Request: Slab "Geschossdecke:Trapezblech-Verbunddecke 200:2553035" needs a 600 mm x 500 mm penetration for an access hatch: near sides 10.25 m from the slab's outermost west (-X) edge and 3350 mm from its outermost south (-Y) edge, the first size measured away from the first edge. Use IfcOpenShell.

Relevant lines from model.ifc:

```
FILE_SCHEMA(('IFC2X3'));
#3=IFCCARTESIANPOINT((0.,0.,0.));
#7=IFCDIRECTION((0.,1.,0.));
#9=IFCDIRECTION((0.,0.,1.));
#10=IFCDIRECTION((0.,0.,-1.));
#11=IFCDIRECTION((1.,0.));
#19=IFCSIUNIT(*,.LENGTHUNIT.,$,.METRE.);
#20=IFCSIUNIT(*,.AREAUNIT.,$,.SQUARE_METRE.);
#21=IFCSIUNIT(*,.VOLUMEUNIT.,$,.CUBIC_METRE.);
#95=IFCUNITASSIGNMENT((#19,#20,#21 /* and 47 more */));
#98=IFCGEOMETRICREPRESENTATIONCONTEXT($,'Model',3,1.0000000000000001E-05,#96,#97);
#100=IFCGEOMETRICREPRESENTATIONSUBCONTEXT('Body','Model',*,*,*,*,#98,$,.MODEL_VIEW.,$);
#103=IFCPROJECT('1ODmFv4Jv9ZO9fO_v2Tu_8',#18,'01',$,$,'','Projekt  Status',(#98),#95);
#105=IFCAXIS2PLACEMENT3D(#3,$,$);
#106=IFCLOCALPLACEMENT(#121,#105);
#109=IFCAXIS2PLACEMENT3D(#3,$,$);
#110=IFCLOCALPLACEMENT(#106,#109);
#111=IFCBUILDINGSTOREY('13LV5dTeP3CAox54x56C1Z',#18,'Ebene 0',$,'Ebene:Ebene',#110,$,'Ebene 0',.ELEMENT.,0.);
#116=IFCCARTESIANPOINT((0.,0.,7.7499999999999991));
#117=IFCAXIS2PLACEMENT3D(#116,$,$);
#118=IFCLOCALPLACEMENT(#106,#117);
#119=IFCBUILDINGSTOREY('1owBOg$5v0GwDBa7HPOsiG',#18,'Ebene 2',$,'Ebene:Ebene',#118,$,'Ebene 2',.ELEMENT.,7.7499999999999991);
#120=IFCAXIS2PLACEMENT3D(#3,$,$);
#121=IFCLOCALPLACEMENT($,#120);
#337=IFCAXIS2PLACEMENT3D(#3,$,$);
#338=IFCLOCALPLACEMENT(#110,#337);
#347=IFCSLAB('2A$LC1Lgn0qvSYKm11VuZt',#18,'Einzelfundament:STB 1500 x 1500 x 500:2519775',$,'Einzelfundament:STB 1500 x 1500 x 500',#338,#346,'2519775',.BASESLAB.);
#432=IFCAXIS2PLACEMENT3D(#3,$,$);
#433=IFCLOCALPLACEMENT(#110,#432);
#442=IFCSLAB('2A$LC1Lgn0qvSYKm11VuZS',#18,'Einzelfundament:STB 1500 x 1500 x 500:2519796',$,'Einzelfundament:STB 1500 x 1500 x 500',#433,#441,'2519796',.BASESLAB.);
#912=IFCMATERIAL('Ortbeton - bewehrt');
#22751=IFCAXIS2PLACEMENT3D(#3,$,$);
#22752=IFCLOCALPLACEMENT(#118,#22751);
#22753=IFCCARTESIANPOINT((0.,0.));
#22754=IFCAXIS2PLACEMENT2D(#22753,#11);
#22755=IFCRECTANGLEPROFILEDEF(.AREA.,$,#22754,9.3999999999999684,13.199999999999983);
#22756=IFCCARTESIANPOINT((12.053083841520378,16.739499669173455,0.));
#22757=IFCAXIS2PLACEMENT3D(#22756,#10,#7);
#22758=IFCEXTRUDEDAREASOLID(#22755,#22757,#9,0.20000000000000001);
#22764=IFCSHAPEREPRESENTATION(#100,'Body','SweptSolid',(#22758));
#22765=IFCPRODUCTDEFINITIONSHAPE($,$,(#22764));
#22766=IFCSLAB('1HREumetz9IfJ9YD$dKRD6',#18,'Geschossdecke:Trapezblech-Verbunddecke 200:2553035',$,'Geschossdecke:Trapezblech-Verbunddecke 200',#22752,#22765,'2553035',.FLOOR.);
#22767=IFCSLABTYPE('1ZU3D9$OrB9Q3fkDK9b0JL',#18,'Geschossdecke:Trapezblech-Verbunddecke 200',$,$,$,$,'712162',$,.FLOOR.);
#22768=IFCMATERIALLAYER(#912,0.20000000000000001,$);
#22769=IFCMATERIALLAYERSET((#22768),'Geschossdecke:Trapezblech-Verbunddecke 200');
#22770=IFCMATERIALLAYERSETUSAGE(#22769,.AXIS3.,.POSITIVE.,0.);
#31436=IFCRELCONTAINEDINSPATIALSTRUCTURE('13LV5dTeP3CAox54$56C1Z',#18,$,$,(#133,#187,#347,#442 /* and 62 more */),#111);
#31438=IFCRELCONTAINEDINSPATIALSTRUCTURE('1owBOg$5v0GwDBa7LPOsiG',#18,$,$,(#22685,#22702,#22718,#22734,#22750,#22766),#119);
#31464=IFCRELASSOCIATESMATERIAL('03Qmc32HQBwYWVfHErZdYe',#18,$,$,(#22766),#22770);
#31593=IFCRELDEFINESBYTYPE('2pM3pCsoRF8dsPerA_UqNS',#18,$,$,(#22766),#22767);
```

```python
import numpy as np
import ifcopenshell
import ifcopenshell.api.feature
import ifcopenshell.api.geometry
import ifcopenshell.api.root
import ifcopenshell.geom
import ifcopenshell.util.placement
import ifcopenshell.util.representation
import ifcopenshell.util.shape
import ifcopenshell.util.unit

model = ifcopenshell.open("model.ifc")
unit_scale = ifcopenshell.util.unit.calculate_unit_scale(model)
settings = ifcopenshell.geom.settings()


def volume(element):
    """Net volume in cubic metres, openings subtracted."""
    shape = ifcopenshell.geom.create_shape(settings, element)
    return ifcopenshell.util.shape.get_volume(shape.geometry)


slab = model.by_guid("1HREumetz9IfJ9YD$dKRD6")
before = volume(slab)

# Extent in the slab's own axes, in metres. The edges named are its -X and -Y sides.
slab_shape = ifcopenshell.geom.create_shape(settings, slab)
vertices = ifcopenshell.util.shape.get_vertices(slab_shape.geometry)
x_min, y_min, bottom = vertices.min(axis=0)
top = vertices[:, 2].max()

opening = ifcopenshell.api.root.create_entity(model, ifc_class="IfcOpeningElement", name="Access hatch opening")
context = ifcopenshell.util.representation.get_context(model, "Model", "Body", "MODEL_VIEW")
width, depth = 0.6, 0.5
outline = [(0.0, 0.0), (width, 0.0), (width, depth), (0.0, depth), (0.0, 0.0)]
# Overshoot both faces by 50 mm so the cut is clean.
shape = ifcopenshell.api.geometry.add_slab_representation(
    model, context=context, depth=top - bottom + 0.1, polyline=outline
)
ifcopenshell.api.geometry.assign_representation(model, product=opening, representation=shape)

matrix = ifcopenshell.util.placement.get_local_placement(slab.ObjectPlacement)
matrix[:, 3] = matrix @ np.append(np.array([x_min + 10.25, y_min + 3.35, bottom - 0.05]) / unit_scale, 1.0)
ifcopenshell.api.geometry.edit_object_placement(model, product=opening, matrix=matrix, is_si=False)
ifcopenshell.api.feature.add_feature(model, feature=opening, element=slab)

after = volume(slab)

print(f"slab volume {before:.3f} -> {after:.3f} m3")

model.write("model_v2.ifc")
```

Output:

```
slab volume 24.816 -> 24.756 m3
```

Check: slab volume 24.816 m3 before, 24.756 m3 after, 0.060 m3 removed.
